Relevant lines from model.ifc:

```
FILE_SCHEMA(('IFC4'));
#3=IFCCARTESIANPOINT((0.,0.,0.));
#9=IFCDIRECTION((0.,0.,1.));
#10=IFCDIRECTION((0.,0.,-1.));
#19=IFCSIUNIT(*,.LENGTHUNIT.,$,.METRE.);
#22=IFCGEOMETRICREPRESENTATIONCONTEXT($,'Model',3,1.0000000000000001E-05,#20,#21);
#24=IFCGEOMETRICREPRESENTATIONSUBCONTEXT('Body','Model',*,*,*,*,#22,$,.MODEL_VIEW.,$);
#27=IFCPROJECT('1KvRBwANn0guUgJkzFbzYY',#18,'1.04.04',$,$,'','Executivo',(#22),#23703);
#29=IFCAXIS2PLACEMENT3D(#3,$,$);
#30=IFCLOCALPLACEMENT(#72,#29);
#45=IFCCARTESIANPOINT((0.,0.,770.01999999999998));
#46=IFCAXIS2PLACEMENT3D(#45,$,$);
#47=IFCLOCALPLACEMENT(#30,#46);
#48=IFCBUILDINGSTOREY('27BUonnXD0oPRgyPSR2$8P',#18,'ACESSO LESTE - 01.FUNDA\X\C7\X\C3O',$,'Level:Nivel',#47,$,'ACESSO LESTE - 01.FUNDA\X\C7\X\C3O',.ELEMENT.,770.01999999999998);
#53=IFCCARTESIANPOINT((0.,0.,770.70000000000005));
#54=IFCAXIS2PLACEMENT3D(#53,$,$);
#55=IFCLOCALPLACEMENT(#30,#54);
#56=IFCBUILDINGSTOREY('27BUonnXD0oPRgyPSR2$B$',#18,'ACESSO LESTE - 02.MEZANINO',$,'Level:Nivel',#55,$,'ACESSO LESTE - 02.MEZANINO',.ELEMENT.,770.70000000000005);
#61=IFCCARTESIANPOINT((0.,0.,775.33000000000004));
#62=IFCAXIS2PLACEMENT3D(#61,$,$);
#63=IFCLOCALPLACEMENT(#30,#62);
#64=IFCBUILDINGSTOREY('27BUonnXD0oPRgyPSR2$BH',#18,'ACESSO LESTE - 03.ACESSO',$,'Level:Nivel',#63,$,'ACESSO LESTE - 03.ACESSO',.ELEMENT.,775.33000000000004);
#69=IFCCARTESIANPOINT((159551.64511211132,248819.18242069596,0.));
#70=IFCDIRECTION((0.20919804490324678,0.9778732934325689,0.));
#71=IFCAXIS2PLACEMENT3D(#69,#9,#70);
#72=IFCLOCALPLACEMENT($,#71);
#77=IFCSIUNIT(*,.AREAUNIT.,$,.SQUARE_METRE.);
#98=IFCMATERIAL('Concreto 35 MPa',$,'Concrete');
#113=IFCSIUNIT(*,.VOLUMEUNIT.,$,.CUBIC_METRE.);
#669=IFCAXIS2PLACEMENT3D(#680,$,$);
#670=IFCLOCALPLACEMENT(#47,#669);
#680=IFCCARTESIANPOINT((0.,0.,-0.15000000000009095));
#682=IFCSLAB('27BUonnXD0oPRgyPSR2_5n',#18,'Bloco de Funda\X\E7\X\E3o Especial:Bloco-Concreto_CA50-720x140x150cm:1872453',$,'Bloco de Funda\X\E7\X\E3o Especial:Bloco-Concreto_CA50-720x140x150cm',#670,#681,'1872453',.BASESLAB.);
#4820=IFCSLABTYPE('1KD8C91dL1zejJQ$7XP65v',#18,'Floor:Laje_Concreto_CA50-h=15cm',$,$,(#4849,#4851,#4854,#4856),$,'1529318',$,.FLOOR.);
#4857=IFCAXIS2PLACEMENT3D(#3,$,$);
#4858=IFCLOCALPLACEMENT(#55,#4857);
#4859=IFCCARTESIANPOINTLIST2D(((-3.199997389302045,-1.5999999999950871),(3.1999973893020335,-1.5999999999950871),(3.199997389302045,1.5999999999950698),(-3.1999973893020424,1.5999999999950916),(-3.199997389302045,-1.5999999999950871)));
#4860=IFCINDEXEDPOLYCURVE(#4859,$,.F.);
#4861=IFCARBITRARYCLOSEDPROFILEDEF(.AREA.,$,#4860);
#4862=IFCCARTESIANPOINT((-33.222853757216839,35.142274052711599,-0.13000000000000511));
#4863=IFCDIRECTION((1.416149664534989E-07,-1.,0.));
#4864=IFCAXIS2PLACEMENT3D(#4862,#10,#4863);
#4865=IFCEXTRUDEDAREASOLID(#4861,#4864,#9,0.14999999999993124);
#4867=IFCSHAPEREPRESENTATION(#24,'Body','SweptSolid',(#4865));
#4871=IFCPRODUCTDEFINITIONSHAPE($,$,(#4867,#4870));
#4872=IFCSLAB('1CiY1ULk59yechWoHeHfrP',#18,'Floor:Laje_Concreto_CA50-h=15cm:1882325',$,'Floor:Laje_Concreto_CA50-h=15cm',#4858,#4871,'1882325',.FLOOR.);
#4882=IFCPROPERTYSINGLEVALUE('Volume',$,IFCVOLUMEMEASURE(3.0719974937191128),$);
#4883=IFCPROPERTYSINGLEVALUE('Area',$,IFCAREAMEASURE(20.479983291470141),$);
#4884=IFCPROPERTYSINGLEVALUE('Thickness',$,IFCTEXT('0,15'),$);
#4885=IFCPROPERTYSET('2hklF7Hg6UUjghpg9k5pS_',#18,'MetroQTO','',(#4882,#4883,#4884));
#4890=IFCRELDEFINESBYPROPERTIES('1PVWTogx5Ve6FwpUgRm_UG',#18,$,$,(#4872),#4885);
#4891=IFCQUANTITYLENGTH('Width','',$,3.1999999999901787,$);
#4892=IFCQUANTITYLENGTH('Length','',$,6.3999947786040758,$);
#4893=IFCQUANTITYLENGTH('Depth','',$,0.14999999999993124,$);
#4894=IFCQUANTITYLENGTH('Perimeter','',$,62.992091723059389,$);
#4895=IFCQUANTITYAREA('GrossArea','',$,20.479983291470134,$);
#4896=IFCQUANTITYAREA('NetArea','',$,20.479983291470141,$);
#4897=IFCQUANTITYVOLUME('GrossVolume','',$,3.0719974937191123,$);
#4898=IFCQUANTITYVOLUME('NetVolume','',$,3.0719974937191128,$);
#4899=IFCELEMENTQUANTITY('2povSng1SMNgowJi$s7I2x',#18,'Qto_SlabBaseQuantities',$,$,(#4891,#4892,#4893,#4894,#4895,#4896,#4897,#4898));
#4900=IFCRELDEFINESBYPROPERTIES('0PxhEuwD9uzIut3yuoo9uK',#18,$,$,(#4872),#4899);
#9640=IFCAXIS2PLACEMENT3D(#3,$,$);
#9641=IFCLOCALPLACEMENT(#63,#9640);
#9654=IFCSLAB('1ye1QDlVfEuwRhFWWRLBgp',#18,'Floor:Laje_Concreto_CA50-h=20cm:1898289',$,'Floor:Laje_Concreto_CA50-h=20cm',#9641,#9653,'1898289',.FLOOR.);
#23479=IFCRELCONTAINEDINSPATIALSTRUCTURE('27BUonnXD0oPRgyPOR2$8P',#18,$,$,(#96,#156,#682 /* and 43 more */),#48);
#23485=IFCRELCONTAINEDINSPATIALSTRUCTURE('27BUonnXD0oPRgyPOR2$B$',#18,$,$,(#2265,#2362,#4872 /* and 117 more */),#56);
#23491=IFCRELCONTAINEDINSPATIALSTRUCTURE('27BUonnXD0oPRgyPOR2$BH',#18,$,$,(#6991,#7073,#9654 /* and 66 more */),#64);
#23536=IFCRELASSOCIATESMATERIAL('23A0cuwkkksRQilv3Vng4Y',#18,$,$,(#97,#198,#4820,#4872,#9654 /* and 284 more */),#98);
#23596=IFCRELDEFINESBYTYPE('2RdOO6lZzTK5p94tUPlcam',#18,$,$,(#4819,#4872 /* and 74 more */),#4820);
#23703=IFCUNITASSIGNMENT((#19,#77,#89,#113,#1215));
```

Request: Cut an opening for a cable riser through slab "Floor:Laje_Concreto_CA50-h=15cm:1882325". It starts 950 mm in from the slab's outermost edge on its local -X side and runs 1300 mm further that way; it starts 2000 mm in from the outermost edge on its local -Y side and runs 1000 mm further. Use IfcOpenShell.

```python
import numpy as np
import ifcopenshell
import ifcopenshell.api.feature
import ifcopenshell.api.geometry
import ifcopenshell.api.pset
import ifcopenshell.api.root
import ifcopenshell.geom
import ifcopenshell.util.element
import ifcopenshell.util.placement
import ifcopenshell.util.representation
import ifcopenshell.util.shape
import ifcopenshell.util.unit

model = ifcopenshell.open("model.ifc")
unit_scale = ifcopenshell.util.unit.calculate_unit_scale(model)
area_scale = ifcopenshell.util.unit.calculate_unit_scale(model, "AREAUNIT")
volume_scale = ifcopenshell.util.unit.calculate_unit_scale(model, "VOLUMEUNIT")
settings = ifcopenshell.geom.settings()


def volume(element):
    """Net volume in cubic metres, openings subtracted."""
    shape = ifcopenshell.geom.create_shape(settings, element)
    return ifcopenshell.util.shape.get_volume(shape.geometry)


slab = model.by_id(4872)
before = volume(slab)

# Extent in the slab's own axes, in metres. The edges named are its -X and -Y sides.
slab_shape = ifcopenshell.geom.create_shape(settings, slab)
vertices = ifcopenshell.util.shape.get_vertices(slab_shape.geometry)
x_min, y_min, bottom = vertices.min(axis=0)
top = vertices[:, 2].max()

opening = ifcopenshell.api.root.create_entity(model, ifc_class="IfcOpeningElement", name="Cable riser opening", predefined_type="OPENING")
context = ifcopenshell.util.representation.get_context(model, "Model", "Body", "MODEL_VIEW")
width, depth = 1.3, 1
outline = [(0.0, 0.0), (width, 0.0), (width, depth), (0.0, depth), (0.0, 0.0)]
# Overshoot both faces by 50 mm so the cut is clean.
shape = ifcopenshell.api.geometry.add_slab_representation(
    model, context=context, depth=top - bottom + 0.1, polyline=outline
)
ifcopenshell.api.geometry.assign_representation(model, product=opening, representation=shape)

matrix = ifcopenshell.util.placement.get_local_placement(slab.ObjectPlacement)
matrix[:, 3] = matrix @ np.append(np.array([x_min + 0.95, y_min + 2, bottom - 0.05]) / unit_scale, 1.0)
ifcopenshell.api.geometry.edit_object_placement(model, product=opening, matrix=matrix, is_si=False)
ifcopenshell.api.feature.add_feature(model, feature=opening, element=slab)

after = volume(slab)

# Update the slab's stored quantities.
pset = model.by_id(ifcopenshell.util.element.get_pset(slab, "MetroQTO", should_inherit=False)["id"])
ifcopenshell.api.pset.edit_pset(model, pset=pset, properties={
    "Volume": model.create_entity("IfcVolumeMeasure", after / volume_scale),
    "Area": model.create_entity("IfcAreaMeasure", after / (top - bottom) / area_scale),
})
qto = model.by_id(ifcopenshell.util.element.get_pset(slab, "Qto_SlabBaseQuantities", should_inherit=False)["id"])
ifcopenshell.api.pset.edit_qto(model, qto=qto, properties={
    "NetArea": after / (top - bottom) / area_scale,
    "NetVolume": after / volume_scale,
})

print(f"slab volume {before:.3f} -> {after:.3f} m3")

model.write("model_updated.ifc")
```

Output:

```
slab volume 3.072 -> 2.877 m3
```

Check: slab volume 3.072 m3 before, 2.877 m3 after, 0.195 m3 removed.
